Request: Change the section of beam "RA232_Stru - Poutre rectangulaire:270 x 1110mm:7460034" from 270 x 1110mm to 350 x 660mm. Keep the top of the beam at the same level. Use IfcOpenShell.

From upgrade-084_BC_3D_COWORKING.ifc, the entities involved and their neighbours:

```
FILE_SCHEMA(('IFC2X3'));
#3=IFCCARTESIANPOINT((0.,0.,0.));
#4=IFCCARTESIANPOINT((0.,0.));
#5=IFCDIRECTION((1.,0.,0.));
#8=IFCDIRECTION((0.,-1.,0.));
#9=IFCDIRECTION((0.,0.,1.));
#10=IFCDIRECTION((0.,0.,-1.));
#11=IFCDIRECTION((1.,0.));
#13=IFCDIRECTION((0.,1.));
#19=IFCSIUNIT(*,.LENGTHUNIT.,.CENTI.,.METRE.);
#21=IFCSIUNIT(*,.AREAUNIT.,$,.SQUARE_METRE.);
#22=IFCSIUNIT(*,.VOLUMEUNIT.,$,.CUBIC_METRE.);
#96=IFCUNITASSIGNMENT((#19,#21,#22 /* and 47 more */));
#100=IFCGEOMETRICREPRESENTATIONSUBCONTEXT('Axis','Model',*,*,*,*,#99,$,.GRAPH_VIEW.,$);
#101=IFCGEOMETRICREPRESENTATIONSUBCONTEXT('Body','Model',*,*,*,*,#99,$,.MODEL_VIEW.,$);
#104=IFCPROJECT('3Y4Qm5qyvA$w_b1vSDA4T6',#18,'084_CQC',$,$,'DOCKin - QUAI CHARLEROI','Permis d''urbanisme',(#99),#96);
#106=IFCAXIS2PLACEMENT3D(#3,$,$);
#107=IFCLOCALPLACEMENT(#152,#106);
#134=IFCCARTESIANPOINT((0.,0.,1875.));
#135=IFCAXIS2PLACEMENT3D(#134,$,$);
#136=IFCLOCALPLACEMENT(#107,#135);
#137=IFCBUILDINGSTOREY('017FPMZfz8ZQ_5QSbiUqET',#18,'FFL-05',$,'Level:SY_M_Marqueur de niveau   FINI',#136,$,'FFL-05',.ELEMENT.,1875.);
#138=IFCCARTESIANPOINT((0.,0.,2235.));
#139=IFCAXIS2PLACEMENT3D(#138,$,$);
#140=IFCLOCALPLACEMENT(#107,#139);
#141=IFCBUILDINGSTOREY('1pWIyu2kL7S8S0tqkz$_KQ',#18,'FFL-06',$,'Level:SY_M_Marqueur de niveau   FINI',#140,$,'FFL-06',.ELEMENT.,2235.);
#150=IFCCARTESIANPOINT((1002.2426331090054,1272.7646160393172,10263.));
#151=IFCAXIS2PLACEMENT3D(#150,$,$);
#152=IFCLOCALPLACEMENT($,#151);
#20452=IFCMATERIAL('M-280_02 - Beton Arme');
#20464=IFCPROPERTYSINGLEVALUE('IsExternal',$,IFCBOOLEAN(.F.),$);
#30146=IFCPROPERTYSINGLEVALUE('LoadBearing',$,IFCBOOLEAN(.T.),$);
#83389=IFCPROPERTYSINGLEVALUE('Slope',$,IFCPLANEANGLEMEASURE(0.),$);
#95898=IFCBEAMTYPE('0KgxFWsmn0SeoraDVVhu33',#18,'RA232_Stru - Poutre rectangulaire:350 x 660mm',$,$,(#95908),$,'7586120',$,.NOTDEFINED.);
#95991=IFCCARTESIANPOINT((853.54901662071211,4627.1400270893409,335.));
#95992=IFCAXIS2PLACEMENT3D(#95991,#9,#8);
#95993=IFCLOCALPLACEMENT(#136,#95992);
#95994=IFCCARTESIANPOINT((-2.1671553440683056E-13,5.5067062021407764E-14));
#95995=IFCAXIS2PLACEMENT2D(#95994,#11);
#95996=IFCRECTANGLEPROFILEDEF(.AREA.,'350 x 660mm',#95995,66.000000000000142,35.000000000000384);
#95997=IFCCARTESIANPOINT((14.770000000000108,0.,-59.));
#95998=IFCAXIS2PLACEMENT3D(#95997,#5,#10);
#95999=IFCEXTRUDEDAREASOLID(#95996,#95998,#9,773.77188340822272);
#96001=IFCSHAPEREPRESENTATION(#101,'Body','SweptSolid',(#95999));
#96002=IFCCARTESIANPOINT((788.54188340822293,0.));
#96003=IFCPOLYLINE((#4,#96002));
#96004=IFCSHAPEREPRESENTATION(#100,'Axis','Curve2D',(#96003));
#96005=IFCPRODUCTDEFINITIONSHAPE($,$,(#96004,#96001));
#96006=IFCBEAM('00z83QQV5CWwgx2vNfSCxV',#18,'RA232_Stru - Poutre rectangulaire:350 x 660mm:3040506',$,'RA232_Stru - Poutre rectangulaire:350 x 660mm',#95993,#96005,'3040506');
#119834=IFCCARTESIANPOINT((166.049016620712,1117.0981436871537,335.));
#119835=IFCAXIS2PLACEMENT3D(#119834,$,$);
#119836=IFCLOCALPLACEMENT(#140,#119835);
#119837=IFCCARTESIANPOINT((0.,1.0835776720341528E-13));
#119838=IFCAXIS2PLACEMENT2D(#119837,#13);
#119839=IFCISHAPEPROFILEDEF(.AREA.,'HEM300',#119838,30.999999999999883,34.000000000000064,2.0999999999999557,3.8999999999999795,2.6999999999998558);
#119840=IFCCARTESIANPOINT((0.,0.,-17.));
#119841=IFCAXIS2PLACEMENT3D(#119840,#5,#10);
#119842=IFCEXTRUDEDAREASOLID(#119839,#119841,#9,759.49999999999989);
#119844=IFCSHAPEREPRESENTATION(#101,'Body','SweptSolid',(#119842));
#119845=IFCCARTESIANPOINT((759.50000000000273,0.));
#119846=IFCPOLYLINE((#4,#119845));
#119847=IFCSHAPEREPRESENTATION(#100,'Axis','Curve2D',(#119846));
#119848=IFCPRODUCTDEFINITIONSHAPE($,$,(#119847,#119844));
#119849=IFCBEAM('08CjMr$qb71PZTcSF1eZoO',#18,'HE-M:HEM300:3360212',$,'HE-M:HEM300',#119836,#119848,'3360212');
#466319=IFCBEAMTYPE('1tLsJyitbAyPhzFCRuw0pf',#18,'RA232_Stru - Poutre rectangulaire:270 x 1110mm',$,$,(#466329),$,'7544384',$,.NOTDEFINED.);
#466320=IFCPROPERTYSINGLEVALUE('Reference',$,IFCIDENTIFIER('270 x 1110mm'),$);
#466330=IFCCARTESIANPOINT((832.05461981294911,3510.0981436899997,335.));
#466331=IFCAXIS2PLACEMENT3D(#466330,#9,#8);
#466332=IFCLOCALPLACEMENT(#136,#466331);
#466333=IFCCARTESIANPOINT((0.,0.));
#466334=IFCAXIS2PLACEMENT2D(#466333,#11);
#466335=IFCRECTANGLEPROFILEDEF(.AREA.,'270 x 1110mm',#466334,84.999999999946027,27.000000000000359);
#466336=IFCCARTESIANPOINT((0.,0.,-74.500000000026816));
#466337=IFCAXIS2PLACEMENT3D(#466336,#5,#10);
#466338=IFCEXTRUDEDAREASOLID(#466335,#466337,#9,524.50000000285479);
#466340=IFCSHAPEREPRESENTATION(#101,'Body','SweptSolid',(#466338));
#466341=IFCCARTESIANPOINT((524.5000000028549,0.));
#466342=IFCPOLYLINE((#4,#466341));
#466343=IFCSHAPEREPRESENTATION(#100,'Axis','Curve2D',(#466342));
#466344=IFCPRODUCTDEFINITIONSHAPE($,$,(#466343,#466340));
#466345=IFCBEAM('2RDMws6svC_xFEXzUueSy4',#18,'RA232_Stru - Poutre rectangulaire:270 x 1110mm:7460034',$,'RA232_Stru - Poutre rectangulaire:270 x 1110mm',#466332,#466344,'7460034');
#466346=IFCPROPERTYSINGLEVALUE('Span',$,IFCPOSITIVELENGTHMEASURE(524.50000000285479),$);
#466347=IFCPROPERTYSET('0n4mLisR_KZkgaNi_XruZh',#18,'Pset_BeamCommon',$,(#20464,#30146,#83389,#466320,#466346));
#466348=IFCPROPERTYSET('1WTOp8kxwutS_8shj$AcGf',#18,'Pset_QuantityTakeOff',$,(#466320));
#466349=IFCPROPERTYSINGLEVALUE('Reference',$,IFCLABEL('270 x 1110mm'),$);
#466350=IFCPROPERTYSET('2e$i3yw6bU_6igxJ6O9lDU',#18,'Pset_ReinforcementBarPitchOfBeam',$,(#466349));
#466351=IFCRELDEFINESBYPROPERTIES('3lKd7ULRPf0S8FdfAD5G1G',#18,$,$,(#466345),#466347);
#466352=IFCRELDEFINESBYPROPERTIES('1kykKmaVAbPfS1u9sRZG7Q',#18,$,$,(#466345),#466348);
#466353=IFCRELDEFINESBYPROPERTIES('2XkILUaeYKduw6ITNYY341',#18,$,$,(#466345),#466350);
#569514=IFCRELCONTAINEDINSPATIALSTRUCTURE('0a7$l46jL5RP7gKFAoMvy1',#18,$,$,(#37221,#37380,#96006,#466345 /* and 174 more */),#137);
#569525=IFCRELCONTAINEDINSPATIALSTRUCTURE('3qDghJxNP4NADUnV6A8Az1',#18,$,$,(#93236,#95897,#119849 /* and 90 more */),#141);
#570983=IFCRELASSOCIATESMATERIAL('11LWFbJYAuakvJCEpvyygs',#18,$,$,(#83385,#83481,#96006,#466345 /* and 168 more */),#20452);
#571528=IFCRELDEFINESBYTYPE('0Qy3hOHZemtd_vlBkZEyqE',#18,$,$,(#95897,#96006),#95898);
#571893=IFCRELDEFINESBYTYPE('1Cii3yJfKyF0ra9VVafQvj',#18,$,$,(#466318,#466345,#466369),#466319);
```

```python
import ifcopenshell
import ifcopenshell.api.pset
import ifcopenshell.api.type
import ifcopenshell.util.element
import ifcopenshell.util.representation

model = ifcopenshell.open("upgrade-084_BC_3D_COWORKING.ifc")

member = model.by_guid("2RDMws6svC_xFEXzUueSy4")
source = next(p for p in model.by_type("IfcRectangleProfileDef") if p.ProfileName == "350 x 660mm")

body = ifcopenshell.util.representation.get_representation(member, "Model", "Body")
solid = body.Items[0]
old_profile = solid.SweptArea

# Copy the section's sizes but keep this member's own profile position.
profile = ifcopenshell.util.element.copy(model, source)
# Profiles are centred, so shift by half the change in depth to hold the top.
shift = (old_profile.XDim - profile.XDim) / 2
x, y = old_profile.Position.Location.Coordinates
up = (-1.0, 0.0)  # upwards, in the solid's own plane
location = model.createIfcCartesianPoint((x + up[0] * shift, y + up[1] * shift))
profile.Position = model.createIfcAxis2Placement2D(location, old_profile.Position.RefDirection)
solid.SweptArea = profile
if not model.get_total_inverses(old_profile):
    ifcopenshell.util.element.remove_deep2(model, old_profile)

new_type = model.by_guid("0KgxFWsmn0SeoraDVVhu33")
ifcopenshell.api.type.assign_type(
    model, related_objects=[member], relating_type=new_type, should_map_representations=False
)
member.Name = member.Name.replace("270 x 1110mm", "350 x 660mm")
member.ObjectType = "RA232_Stru - Poutre rectangulaire:350 x 660mm"
pset = model.by_id(ifcopenshell.util.element.get_pset(member, "Pset_BeamCommon", should_inherit=False)["id"])
ifcopenshell.api.pset.edit_pset(model, pset=pset, properties={"Reference": "350 x 660mm"})
pset = model.by_id(ifcopenshell.util.element.get_pset(member, "Pset_QuantityTakeOff", should_inherit=False)["id"])
ifcopenshell.api.pset.edit_pset(model, pset=pset, properties={"Reference": "350 x 660mm"})
pset = model.by_id(ifcopenshell.util.element.get_pset(member, "Pset_ReinforcementBarPitchOfBeam", should_inherit=False)["id"])
ifcopenshell.api.pset.edit_pset(model, pset=pset, properties={"Reference": "350 x 660mm"})

print(solid.SweptArea)

model.write("upgrade-084_BC_3D_COWORKING_v2.ifc")
```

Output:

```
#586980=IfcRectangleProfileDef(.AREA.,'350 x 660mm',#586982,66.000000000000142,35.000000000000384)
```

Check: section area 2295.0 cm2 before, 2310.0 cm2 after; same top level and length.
